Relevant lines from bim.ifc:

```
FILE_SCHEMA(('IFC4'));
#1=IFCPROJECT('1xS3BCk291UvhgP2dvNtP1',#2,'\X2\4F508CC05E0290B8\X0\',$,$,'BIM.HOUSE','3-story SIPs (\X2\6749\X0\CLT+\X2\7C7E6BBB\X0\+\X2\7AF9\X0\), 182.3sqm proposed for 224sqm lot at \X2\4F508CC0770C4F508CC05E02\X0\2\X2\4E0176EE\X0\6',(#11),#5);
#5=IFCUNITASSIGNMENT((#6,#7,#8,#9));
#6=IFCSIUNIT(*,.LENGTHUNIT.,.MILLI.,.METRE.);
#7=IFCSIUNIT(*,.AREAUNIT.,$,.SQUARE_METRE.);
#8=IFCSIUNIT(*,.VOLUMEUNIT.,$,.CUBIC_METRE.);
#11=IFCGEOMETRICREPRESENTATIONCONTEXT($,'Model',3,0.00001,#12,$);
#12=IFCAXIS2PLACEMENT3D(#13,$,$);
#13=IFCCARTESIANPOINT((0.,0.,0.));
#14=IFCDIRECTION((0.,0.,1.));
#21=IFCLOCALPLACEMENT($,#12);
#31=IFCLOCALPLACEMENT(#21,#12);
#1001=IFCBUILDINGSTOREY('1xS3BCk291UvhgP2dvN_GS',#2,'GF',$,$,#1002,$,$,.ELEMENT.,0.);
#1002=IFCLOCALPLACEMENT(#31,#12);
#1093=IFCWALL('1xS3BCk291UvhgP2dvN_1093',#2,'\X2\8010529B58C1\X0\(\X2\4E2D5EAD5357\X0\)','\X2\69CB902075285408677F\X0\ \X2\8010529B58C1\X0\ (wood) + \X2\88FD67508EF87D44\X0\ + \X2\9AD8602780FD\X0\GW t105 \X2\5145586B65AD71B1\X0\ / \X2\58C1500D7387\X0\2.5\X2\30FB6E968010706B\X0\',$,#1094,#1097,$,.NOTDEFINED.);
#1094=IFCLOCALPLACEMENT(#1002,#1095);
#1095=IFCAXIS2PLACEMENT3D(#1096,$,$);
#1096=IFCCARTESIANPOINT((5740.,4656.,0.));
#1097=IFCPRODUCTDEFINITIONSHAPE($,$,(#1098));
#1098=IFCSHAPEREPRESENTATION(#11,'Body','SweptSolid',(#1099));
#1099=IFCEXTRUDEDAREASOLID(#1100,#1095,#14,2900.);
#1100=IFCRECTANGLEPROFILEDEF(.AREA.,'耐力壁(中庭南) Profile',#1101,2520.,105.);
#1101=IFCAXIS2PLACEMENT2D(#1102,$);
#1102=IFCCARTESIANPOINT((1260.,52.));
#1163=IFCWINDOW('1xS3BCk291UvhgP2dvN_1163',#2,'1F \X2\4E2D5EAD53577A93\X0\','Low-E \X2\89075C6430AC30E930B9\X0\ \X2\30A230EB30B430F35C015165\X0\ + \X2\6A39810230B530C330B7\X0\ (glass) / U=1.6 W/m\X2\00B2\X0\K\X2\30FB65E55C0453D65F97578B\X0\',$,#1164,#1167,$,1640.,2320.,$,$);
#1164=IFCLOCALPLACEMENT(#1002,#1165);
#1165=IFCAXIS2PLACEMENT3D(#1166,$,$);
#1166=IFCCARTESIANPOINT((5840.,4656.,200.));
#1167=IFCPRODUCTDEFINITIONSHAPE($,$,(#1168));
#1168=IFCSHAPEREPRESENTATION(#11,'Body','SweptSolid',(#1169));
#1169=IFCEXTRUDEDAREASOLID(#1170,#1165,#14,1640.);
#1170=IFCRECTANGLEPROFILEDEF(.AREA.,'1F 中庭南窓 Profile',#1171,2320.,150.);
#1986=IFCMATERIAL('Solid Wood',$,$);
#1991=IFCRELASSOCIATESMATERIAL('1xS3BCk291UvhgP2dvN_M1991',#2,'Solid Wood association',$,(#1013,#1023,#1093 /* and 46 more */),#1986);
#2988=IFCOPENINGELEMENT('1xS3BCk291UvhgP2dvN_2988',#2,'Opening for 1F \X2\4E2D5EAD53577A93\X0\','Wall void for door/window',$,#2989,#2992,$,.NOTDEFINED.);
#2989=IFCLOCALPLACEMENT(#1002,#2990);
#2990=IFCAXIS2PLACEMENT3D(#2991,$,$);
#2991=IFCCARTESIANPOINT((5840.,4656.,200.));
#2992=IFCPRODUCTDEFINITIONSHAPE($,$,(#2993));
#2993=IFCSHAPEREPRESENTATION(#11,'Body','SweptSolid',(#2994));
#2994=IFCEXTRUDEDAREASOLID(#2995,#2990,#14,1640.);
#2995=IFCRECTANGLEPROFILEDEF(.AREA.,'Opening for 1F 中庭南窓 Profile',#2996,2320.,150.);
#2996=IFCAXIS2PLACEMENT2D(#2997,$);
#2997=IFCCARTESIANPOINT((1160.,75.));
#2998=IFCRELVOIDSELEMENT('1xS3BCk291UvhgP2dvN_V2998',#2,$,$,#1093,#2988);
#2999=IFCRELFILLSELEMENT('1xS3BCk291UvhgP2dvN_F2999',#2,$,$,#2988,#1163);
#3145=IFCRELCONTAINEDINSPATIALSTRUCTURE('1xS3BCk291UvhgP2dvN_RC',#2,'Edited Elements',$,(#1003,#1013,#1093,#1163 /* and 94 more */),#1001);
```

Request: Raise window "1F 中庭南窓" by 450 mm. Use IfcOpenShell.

```python
import numpy as np
import ifcopenshell
import ifcopenshell.api.geometry
import ifcopenshell.util.placement
import ifcopenshell.util.unit

model = ifcopenshell.open("bim.ifc")
unit_scale = ifcopenshell.util.unit.calculate_unit_scale(model)

window = model.by_guid("1xS3BCk291UvhgP2dvN_1163")
opening = window.FillsVoids[0].RelatingOpeningElement
dz = 0.45 / unit_scale

shift = np.array([0.0, 0.0, dz])
# The window is not placed relative to its opening, so move both.
for product in (opening, window):
    matrix = ifcopenshell.util.placement.get_local_placement(product.ObjectPlacement)
    matrix[:3, 3] += shift
    ifcopenshell.api.geometry.edit_object_placement(model, product=product, matrix=matrix, is_si=False)

print(f"moved by {dz * unit_scale:+.3f} m")

model.write("bim_rev.ifc")
```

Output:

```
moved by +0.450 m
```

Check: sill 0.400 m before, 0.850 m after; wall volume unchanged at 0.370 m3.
